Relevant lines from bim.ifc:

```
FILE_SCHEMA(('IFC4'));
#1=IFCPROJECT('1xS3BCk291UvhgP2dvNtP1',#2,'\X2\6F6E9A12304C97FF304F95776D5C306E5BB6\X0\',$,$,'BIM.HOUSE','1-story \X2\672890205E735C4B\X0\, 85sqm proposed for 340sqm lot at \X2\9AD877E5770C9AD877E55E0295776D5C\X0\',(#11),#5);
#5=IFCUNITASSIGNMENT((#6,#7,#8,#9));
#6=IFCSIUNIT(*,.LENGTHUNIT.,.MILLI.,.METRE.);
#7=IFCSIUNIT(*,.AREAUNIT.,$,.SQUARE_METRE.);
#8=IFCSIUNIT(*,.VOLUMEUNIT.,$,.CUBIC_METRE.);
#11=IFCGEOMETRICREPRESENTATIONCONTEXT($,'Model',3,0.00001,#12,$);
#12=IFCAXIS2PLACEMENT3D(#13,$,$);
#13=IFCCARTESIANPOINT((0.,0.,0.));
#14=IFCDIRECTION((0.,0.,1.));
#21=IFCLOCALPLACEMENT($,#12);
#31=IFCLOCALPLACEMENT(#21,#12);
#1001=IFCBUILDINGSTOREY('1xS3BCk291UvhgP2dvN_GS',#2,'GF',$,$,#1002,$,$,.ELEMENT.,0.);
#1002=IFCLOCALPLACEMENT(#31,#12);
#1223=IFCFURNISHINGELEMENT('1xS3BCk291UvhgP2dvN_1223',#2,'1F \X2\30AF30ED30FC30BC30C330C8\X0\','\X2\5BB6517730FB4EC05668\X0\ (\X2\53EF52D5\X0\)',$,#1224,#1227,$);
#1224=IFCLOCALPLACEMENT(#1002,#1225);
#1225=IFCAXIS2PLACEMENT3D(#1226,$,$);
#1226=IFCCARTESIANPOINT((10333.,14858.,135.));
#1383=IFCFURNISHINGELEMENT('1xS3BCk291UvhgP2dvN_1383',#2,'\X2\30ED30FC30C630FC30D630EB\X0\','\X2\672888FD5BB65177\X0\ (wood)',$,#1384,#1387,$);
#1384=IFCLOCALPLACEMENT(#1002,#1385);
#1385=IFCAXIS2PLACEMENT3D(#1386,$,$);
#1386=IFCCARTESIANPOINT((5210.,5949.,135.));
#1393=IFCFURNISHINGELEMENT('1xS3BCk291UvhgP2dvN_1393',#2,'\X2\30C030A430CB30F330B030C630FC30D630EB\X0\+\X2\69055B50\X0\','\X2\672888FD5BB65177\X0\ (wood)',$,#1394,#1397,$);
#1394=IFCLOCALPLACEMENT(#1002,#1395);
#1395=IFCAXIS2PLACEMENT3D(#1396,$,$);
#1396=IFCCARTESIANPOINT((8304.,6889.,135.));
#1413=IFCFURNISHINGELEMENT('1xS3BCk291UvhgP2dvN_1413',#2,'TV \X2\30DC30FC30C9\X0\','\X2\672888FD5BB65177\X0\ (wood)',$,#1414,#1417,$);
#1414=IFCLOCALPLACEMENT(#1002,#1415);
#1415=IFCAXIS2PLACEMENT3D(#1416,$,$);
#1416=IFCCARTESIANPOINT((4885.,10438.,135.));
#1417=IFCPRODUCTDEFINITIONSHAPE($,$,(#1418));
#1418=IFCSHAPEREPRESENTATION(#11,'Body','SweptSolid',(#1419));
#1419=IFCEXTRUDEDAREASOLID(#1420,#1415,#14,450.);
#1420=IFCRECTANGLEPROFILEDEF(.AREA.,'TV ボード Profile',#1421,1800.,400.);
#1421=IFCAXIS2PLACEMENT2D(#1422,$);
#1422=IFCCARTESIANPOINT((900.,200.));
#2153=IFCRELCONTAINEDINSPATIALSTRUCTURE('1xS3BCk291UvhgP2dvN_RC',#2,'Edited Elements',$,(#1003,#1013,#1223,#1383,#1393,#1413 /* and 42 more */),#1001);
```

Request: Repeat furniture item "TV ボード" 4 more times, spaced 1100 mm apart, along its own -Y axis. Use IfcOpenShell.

```python
import ifcopenshell
import ifcopenshell.api.geometry
import ifcopenshell.api.root
import ifcopenshell.util.element
import ifcopenshell.util.placement

model = ifcopenshell.open("bim.ifc")


def reuse_history(source, copy):
    """copy_class also copies each property set's owner history, people and application; keep the originals."""
    for rel in copy.IsDefinedBy:
        if rel.is_a("IfcRelDefinesByProperties") and (history := rel.RelatingPropertyDefinition.OwnerHistory):
            rel.RelatingPropertyDefinition.OwnerHistory = source.OwnerHistory
            ifcopenshell.util.element.remove_deep2(model, history)


source = model.by_guid("1xS3BCk291UvhgP2dvN_1413")
base = ifcopenshell.util.placement.get_local_placement(source.ObjectPlacement)
step = -base[:3, 1] * 1100.0

for i in range(1, 5):
    copy = ifcopenshell.api.root.copy_class(model, product=source)
    copy.Representation = ifcopenshell.util.element.copy_deep(
        model, source.Representation, exclude=["IfcGeometricRepresentationContext", "IfcRepresentationMap"]
    )
    reuse_history(source, copy)
    matrix = base.copy()
    matrix[:3, 3] += i * step
    print("added at", matrix[:3, 3].round(3) + 0.0)
    ifcopenshell.api.geometry.edit_object_placement(model, product=copy, matrix=matrix, is_si=False)

model.write("bim_updated.ifc")
```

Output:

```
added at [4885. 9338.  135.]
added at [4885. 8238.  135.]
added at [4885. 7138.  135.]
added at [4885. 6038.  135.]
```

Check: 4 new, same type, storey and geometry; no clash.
